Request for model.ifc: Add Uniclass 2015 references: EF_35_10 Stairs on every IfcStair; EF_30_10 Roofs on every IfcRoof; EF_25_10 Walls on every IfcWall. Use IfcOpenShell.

First a look at what the model holds.

```python
import ifcopenshell

model = ifcopenshell.open("model.ifc")
print(model.schema)
print("classifications:", [c.Name for c in model.by_type("IfcClassification")])
for ifc_class in ("IfcDoor", "IfcRoof", "IfcStair", "IfcWall", "IfcWindow"):
    print(ifc_class, len(model.by_type(ifc_class)))
```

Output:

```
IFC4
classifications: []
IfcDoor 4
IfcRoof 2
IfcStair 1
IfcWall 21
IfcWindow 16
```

```python
import ifcopenshell
import ifcopenshell.api.classification

model = ifcopenshell.open("model.ifc")

system = ifcopenshell.api.classification.add_classification(model, classification="Uniclass 2015")

codes = {
    "IfcStair": ("EF_35_10", "Stairs"),
    "IfcRoof": ("EF_30_10", "Roofs"),
    "IfcWall": ("EF_25_10", "Walls"),
}
for ifc_class, (code, name) in codes.items():
    products = model.by_type(ifc_class)
    ifcopenshell.api.classification.add_reference(
        model, products=products, classification=system, identification=code, name=name
    )
    print(code, len(products))

model.write("model_rev.ifc")
```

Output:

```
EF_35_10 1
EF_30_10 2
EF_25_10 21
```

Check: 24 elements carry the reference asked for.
